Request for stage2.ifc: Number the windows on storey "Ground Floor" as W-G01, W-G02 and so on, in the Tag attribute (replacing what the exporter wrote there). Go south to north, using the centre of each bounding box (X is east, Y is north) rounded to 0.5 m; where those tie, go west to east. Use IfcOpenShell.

First a look at what the model holds.

```python
import ifcopenshell
import ifcopenshell.util.element
import ifcopenshell.util.placement

model = ifcopenshell.open("stage2.ifc")
print(model.schema)
storey = next(s for s in model.by_type("IfcBuildingStorey") if s.Name == "Ground Floor")
windows = [e for e in ifcopenshell.util.element.get_decomposition(storey) if e.is_a("IfcWindow")]
for e in sorted(windows, key=lambda e: e.id()):
    origin = ifcopenshell.util.placement.get_local_placement(e.ObjectPlacement)[:3, 3]
    print(e.id(), e.Tag, e.Name, origin.round(2) + 0.0, sep=" | ")
```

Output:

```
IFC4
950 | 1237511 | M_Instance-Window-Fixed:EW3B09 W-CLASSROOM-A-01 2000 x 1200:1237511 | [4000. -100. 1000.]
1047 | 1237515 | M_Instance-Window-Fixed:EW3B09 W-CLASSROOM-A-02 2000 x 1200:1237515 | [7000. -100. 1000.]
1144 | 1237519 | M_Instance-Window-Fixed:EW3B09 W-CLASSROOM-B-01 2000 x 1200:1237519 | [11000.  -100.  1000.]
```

```python
import ifcopenshell
import ifcopenshell.geom
import ifcopenshell.util.element
import ifcopenshell.util.shape

model = ifcopenshell.open("stage2.ifc")
settings = ifcopenshell.geom.settings()
settings.set("use-world-coords", True)


def centre(element):
    shape = ifcopenshell.geom.create_shape(settings, element)
    return ifcopenshell.util.shape.get_bbox_centroid(shape.geometry)


storey = next(s for s in model.by_type("IfcBuildingStorey") if s.Name == "Ground Floor")
windows = [e for e in ifcopenshell.util.element.get_decomposition(storey) if e.is_a("IfcWindow")]

# Insertion points can sit at a corner or the storey origin, so sort by the geometry (in metres).
centres = {e: centre(e) for e in windows}
windows.sort(key=lambda e: (round(centres[e][1] / 0.5), centres[e][0]))

for i, e in enumerate(windows, start=1):
    number = f"W-G{i:02d}"
    e.Tag = number
    print(e.id(), number)

model.write("stage2_v2.ifc")
```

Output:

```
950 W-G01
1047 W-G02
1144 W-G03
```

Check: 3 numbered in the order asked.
